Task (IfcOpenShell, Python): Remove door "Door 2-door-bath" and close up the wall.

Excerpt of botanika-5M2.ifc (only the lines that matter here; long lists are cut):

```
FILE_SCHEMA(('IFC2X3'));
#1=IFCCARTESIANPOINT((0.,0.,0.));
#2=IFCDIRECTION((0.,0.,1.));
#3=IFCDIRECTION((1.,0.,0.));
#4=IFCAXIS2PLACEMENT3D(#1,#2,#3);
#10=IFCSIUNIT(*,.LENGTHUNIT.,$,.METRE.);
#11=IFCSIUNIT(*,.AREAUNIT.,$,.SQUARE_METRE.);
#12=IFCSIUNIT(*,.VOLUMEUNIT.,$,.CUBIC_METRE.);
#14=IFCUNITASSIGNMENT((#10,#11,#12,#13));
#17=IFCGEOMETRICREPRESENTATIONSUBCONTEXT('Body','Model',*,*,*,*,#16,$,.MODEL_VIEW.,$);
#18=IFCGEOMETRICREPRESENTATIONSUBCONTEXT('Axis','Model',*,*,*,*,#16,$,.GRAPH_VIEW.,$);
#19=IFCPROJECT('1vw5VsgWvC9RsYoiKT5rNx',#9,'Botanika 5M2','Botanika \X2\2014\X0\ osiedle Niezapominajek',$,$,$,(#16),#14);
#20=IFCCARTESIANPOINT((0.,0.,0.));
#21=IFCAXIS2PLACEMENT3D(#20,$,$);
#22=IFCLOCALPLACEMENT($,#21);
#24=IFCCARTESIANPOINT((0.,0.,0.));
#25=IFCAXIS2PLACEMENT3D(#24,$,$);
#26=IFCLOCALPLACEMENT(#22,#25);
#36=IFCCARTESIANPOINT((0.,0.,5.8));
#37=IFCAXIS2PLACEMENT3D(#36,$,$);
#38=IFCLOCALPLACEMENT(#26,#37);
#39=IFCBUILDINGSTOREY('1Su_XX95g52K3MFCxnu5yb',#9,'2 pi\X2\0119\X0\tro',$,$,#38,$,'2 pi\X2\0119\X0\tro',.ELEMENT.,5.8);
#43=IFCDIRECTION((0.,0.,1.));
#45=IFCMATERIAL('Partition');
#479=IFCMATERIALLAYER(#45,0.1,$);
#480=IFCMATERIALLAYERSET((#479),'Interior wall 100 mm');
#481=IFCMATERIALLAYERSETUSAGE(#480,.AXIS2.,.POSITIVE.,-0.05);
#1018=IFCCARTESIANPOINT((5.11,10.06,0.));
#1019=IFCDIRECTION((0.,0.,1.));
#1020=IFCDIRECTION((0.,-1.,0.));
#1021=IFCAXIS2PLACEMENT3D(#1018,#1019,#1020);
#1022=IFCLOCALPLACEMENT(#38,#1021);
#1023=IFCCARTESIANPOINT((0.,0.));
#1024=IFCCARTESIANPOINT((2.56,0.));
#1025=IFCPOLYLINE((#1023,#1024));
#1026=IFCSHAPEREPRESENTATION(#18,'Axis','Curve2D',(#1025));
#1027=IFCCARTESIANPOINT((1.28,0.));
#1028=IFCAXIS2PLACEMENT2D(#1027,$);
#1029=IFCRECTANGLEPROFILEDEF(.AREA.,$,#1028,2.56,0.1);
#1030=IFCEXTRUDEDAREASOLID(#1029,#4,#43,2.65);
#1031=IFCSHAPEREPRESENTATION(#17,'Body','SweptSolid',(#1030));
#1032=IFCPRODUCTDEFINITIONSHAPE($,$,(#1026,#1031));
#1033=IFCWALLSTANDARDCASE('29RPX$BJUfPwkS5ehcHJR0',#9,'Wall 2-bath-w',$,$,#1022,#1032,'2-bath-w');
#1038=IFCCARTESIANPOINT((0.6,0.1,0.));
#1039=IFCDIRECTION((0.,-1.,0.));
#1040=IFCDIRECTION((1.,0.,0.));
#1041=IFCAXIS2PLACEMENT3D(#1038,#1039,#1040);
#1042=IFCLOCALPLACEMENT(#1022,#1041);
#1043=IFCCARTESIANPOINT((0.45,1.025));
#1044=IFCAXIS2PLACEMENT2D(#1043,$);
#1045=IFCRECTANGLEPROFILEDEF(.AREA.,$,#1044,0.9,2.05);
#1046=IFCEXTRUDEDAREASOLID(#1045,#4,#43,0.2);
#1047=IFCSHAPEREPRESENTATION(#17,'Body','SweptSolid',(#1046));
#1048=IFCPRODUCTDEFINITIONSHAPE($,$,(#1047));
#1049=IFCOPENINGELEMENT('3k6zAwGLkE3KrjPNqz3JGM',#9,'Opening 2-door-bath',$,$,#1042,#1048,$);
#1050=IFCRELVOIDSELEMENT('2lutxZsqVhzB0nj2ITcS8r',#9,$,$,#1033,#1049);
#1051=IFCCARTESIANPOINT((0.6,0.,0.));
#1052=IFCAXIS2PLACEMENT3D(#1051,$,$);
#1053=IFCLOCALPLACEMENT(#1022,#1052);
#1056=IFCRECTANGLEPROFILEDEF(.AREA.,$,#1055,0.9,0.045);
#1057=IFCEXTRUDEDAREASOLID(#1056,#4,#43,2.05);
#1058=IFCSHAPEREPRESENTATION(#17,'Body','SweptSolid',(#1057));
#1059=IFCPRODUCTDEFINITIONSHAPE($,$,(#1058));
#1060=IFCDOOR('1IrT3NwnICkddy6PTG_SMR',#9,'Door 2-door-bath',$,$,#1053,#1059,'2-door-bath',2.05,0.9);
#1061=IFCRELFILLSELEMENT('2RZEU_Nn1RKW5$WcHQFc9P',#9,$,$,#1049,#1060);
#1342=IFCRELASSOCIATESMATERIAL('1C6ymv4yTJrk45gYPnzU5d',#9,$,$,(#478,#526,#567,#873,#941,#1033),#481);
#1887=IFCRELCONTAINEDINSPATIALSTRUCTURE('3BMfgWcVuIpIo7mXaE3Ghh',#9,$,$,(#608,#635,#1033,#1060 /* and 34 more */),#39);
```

```python
import ifcopenshell
import ifcopenshell.api.feature
import ifcopenshell.api.root
import ifcopenshell.geom
import ifcopenshell.util.shape

model = ifcopenshell.open("botanika-5M2.ifc")
settings = ifcopenshell.geom.settings()


def volume(element):
    """Net volume in cubic metres, openings subtracted."""
    shape = ifcopenshell.geom.create_shape(settings, element)
    return ifcopenshell.util.shape.get_volume(shape.geometry)


door = model.by_guid("1IrT3NwnICkddy6PTG_SMR")
opening = door.FillsVoids[0].RelatingOpeningElement
wall = opening.VoidsElements[0].RelatingBuildingElement
before = volume(wall)

ifcopenshell.api.root.remove_product(model, product=door)
ifcopenshell.api.feature.remove_feature(model, feature=opening)

after = volume(wall)

print(f"wall volume {before:.3f} -> {after:.3f} m3")

model.write("botanika-5M2_rev.ifc")
```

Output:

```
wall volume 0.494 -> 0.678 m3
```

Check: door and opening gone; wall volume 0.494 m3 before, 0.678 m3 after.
